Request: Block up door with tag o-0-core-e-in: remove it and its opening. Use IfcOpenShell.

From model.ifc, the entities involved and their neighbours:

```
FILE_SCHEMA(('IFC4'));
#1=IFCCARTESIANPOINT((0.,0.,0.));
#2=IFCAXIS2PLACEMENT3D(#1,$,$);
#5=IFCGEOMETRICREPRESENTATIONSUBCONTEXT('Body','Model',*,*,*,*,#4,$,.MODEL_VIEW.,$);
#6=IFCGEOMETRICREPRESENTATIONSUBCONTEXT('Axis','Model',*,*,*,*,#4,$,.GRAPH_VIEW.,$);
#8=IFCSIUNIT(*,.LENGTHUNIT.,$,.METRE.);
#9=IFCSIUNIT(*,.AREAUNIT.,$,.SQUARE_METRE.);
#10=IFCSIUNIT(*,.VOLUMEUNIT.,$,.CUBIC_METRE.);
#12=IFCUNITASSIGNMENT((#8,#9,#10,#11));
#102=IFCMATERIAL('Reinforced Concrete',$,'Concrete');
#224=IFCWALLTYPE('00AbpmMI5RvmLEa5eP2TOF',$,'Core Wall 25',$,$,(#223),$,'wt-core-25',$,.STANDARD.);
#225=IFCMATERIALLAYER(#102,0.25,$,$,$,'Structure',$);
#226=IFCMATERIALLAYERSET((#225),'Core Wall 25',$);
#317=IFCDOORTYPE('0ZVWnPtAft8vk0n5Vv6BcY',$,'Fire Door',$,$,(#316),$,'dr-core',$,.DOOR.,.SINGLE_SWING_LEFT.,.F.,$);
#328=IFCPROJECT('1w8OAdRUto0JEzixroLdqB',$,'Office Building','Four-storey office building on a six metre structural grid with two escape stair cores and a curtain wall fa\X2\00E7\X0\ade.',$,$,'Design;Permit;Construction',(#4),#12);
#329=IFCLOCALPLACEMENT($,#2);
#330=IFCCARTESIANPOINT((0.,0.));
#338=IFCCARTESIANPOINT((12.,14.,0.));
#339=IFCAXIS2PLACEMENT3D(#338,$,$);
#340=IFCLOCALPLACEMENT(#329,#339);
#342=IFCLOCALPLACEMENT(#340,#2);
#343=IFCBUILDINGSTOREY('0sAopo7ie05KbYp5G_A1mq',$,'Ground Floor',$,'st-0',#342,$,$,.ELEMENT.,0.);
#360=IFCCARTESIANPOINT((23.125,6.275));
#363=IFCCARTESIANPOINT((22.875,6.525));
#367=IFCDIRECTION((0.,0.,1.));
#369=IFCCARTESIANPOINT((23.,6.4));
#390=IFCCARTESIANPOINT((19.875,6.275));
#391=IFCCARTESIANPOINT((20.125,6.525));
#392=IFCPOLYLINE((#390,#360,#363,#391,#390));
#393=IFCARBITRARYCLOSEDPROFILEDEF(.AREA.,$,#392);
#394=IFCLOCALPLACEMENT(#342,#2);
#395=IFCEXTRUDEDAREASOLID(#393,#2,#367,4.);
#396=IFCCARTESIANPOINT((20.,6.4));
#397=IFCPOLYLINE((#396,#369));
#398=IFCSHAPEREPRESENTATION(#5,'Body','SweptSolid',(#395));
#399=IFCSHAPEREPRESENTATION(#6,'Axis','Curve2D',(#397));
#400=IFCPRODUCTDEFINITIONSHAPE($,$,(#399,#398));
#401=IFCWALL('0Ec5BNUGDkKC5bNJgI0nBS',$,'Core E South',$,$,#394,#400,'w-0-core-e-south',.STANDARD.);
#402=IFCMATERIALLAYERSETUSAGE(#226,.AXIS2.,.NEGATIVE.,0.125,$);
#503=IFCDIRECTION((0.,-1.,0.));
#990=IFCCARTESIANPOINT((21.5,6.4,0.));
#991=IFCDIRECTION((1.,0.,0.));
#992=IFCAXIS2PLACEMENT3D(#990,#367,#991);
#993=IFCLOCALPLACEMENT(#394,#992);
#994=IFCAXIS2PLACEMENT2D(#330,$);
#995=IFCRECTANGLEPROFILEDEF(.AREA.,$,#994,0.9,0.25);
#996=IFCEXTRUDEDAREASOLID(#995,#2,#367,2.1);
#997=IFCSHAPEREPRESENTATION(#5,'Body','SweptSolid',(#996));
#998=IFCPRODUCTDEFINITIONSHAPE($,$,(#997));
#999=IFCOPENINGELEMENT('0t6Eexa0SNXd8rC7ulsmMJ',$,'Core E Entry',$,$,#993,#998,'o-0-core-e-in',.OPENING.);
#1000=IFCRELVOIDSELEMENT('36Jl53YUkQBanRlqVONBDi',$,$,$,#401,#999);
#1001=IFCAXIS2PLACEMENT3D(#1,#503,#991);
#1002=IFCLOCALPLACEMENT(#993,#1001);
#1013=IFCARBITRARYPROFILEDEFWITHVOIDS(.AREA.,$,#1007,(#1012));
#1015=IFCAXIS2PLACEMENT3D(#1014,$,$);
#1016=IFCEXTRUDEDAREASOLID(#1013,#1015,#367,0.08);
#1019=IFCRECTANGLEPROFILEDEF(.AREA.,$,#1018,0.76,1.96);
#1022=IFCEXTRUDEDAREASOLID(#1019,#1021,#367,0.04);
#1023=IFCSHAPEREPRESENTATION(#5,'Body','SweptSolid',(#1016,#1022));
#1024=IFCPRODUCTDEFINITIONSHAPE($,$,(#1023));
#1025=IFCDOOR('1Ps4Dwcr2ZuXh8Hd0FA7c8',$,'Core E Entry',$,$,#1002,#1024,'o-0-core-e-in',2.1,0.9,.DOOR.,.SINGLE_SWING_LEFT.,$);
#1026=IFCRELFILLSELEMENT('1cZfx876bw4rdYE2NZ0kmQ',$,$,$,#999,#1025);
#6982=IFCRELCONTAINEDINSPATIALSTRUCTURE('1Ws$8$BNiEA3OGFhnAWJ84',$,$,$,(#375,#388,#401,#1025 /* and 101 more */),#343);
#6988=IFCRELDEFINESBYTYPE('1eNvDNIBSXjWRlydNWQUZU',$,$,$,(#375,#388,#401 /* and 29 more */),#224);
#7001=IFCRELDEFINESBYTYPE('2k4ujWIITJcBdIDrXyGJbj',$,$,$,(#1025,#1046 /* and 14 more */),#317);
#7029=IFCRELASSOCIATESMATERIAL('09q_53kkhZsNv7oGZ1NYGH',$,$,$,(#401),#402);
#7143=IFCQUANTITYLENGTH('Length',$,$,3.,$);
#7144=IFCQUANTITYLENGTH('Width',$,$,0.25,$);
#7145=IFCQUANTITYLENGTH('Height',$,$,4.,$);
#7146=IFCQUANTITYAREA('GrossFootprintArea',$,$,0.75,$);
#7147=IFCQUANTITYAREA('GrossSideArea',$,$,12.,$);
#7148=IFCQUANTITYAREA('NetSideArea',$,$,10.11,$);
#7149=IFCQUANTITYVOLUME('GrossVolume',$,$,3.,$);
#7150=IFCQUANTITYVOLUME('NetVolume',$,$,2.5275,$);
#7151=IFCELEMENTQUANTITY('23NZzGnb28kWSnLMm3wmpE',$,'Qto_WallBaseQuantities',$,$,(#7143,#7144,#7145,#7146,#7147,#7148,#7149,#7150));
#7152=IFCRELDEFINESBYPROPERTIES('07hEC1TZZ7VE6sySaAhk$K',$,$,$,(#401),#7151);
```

```python
import ifcopenshell
import ifcopenshell.api.feature
import ifcopenshell.api.pset
import ifcopenshell.api.root
import ifcopenshell.geom
import ifcopenshell.util.element
import ifcopenshell.util.shape
import ifcopenshell.util.unit

model = ifcopenshell.open("model.ifc")
area_scale = ifcopenshell.util.unit.calculate_unit_scale(model, "AREAUNIT")
volume_scale = ifcopenshell.util.unit.calculate_unit_scale(model, "VOLUMEUNIT")
settings = ifcopenshell.geom.settings()


def volume(element):
    """Net volume in cubic metres, openings subtracted."""
    shape = ifcopenshell.geom.create_shape(settings, element)
    return ifcopenshell.util.shape.get_volume(shape.geometry)


door = model.by_guid("1Ps4Dwcr2ZuXh8Hd0FA7c8")
opening = door.FillsVoids[0].RelatingOpeningElement
wall = opening.VoidsElements[0].RelatingBuildingElement
before = volume(wall)

ifcopenshell.api.root.remove_product(model, product=door)
ifcopenshell.api.feature.remove_feature(model, feature=opening)

after = volume(wall)
thickness = 0.25  # wall thickness in metres

# Update the wall's stored quantities.
qto = model.by_id(ifcopenshell.util.element.get_pset(wall, "Qto_WallBaseQuantities", should_inherit=False)["id"])
ifcopenshell.api.pset.edit_qto(model, qto=qto, properties={
    "NetSideArea": after / thickness / area_scale,
    "NetVolume": after / volume_scale,
})

print(f"wall volume {before:.3f} -> {after:.3f} m3")

model.write("model_updated.ifc")
```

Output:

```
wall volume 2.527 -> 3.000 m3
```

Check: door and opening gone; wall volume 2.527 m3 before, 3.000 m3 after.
